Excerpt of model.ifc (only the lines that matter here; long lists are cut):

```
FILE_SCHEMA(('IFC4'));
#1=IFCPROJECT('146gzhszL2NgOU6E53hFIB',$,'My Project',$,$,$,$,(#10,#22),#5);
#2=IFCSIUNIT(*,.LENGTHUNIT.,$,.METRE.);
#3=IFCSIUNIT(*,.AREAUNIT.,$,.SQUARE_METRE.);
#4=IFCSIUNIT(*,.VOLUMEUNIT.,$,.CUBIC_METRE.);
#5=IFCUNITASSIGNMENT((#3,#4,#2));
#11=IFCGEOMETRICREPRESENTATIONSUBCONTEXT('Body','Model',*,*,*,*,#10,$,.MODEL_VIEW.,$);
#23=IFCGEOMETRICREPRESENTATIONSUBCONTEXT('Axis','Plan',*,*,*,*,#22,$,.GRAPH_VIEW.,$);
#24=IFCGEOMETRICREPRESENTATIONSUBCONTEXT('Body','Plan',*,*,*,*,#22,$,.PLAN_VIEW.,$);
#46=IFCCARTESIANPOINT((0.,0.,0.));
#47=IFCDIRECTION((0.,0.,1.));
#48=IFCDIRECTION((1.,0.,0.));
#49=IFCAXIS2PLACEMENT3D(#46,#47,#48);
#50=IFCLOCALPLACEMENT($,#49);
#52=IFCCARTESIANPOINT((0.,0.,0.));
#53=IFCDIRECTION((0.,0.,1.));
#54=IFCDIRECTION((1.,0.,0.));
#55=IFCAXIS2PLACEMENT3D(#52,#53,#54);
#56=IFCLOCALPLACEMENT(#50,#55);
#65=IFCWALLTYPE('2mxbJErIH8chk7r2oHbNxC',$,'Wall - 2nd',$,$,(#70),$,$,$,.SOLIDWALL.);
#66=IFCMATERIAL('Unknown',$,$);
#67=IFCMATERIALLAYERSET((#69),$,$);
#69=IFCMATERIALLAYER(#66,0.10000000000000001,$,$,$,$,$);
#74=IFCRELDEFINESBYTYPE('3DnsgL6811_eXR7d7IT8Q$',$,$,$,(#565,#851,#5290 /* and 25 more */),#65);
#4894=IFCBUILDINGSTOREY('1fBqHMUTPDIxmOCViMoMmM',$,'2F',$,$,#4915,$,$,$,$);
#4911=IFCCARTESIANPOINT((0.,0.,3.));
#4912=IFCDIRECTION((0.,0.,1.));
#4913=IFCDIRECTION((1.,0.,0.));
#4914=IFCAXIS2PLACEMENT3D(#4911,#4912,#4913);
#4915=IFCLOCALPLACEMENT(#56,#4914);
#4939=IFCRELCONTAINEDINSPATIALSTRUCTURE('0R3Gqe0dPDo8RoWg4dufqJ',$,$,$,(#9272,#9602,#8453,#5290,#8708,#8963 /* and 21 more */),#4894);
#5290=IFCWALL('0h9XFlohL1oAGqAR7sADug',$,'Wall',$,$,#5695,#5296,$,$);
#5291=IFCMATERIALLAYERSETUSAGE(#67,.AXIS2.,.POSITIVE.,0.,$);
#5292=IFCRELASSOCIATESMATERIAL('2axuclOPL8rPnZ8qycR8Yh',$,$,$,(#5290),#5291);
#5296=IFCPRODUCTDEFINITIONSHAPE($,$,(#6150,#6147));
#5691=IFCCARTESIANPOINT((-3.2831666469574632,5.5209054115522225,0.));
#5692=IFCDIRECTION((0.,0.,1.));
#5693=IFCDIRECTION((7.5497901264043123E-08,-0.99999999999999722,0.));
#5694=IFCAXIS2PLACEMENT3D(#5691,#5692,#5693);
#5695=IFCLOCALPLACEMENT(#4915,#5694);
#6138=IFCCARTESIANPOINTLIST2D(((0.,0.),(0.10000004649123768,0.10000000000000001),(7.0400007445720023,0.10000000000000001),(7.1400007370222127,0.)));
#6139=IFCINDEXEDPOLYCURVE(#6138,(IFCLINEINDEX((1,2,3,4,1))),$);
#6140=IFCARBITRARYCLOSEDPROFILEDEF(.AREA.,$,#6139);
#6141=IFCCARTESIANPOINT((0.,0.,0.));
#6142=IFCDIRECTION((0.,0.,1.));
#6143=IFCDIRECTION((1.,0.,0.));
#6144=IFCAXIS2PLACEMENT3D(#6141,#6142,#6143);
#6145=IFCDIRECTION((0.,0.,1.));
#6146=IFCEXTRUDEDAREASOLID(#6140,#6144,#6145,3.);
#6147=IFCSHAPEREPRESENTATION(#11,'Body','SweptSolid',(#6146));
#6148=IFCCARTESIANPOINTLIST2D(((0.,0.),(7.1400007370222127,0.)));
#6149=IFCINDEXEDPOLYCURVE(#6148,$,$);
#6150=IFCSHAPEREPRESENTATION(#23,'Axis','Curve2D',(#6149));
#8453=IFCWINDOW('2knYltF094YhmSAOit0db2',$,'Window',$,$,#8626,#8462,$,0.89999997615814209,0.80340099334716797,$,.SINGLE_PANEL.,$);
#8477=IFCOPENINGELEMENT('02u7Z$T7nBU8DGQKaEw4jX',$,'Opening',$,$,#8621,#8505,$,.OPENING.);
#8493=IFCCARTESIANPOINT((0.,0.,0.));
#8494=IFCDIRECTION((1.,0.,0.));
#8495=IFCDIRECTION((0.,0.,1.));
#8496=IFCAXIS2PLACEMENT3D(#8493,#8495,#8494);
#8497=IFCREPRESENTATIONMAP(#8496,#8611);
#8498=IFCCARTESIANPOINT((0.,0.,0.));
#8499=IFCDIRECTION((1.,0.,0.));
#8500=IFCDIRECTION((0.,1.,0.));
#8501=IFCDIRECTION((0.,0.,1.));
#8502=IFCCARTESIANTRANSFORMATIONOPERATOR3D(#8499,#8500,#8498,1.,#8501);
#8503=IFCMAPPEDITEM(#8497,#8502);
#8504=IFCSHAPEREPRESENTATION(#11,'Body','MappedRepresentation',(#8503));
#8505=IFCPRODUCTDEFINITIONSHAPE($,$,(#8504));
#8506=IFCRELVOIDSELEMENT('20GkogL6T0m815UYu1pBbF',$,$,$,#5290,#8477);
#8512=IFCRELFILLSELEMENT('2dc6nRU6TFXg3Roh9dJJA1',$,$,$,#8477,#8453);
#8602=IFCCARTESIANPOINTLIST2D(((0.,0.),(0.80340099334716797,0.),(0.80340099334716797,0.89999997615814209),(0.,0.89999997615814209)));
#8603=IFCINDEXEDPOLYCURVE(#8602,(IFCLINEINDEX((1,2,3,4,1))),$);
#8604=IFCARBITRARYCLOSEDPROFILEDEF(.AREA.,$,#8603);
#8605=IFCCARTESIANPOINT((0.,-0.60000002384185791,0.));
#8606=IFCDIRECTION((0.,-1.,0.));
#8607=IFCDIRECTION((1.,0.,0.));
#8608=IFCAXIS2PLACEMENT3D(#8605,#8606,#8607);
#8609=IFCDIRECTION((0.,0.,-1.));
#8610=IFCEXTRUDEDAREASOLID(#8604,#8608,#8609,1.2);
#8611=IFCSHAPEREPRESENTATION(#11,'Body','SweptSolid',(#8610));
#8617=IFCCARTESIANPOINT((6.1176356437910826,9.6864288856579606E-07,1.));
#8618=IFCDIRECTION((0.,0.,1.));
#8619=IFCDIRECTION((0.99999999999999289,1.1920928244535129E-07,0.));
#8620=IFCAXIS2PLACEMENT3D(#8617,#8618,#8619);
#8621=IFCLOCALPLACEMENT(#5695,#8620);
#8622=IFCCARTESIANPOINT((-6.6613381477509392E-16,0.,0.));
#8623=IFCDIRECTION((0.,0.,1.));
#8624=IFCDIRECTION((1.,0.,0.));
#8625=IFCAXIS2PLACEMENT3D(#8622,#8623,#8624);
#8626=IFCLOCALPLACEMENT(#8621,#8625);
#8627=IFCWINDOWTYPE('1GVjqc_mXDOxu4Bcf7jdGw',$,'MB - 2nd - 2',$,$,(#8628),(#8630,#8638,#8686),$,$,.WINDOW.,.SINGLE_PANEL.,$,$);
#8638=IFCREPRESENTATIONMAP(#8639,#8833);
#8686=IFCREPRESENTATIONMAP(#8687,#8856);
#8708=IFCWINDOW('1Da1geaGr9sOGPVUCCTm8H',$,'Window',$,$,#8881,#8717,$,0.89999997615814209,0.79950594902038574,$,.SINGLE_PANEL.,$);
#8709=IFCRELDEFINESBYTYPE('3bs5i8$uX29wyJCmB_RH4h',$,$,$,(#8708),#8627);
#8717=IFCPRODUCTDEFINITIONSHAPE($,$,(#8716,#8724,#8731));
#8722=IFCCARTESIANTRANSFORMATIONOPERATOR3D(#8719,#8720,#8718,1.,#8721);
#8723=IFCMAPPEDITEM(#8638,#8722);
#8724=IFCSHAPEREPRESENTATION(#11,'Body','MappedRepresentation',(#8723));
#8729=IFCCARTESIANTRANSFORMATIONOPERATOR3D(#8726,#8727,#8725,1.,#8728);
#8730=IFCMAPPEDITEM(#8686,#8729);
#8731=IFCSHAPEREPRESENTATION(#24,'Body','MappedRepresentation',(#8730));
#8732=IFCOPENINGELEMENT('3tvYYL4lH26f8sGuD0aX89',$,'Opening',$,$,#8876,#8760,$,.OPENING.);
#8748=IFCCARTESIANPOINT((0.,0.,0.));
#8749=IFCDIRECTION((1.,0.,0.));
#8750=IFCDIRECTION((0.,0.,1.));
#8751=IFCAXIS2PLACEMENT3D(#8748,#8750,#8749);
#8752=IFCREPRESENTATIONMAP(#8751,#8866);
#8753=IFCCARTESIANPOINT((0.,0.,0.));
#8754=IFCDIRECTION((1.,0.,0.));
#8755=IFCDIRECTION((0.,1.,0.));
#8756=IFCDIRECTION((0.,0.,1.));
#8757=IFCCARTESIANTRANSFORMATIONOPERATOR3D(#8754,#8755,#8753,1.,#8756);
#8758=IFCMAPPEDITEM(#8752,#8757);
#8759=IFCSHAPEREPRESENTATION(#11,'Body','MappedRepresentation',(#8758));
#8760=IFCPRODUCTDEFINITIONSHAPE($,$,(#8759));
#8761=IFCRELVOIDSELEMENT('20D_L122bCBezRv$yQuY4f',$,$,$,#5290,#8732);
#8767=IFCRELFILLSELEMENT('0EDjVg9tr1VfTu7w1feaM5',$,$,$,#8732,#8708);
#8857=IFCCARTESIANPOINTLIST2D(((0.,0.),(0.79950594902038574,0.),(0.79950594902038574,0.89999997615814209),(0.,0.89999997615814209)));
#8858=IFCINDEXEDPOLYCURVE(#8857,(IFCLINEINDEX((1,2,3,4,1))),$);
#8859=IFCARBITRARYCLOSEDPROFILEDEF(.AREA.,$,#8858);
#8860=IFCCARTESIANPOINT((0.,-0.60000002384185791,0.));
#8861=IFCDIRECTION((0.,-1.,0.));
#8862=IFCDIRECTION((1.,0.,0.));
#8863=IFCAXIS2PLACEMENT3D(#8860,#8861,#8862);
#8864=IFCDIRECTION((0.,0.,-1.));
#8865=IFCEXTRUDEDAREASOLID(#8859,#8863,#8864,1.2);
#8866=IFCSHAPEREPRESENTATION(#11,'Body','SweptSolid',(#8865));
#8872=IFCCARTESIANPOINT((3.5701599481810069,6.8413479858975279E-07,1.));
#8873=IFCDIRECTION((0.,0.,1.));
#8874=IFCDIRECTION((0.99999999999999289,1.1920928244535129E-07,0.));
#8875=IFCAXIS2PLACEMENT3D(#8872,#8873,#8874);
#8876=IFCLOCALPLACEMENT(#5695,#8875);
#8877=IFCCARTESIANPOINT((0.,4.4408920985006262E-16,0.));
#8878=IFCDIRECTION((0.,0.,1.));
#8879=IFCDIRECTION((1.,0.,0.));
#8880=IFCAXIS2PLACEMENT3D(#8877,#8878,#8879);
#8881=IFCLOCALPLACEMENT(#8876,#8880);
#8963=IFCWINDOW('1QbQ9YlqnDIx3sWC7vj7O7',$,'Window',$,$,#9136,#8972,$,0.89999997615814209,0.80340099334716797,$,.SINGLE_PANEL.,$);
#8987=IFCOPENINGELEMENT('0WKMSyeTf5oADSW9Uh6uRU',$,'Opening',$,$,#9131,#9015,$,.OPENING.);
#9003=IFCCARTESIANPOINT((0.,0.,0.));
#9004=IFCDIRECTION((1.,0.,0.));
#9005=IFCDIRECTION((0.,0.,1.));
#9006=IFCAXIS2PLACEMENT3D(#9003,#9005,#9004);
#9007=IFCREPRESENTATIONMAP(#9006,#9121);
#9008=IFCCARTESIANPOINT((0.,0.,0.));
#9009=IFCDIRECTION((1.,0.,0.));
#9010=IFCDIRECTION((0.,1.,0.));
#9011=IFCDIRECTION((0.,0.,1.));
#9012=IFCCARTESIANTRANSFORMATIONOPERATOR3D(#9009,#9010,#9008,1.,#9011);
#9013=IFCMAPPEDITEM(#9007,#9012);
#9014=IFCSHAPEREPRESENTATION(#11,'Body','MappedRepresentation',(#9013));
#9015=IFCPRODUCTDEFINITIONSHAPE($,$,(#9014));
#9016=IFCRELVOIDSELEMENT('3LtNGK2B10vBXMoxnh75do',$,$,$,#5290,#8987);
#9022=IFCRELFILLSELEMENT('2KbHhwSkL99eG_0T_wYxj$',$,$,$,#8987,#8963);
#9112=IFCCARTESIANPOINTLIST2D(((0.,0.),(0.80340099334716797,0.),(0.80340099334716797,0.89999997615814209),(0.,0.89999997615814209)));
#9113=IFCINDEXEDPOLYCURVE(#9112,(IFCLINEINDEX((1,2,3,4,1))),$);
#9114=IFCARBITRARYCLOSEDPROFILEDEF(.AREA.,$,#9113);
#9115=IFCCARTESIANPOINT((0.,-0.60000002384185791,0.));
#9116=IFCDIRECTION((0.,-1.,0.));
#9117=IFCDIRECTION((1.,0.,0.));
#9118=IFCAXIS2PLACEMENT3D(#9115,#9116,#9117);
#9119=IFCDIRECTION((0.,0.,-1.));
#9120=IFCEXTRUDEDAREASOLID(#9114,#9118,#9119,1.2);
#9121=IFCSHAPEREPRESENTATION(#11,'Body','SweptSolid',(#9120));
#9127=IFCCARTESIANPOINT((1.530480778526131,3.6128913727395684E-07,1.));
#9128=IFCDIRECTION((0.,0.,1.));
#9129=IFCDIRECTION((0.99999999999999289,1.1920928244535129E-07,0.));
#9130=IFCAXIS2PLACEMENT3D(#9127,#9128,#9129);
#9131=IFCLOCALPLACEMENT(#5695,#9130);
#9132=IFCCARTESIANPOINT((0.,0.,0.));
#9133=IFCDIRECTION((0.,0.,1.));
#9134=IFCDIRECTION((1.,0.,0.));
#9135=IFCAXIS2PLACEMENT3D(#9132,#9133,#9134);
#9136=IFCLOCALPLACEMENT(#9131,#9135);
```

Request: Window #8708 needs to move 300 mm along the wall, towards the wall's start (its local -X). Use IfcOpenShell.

```python
import ifcopenshell
import ifcopenshell.api.geometry
import ifcopenshell.util.placement
import ifcopenshell.util.unit

model = ifcopenshell.open("model.ifc")
unit_scale = ifcopenshell.util.unit.calculate_unit_scale(model)

window = model.by_guid("1Da1geaGr9sOGPVUCCTm8H")
opening = window.FillsVoids[0].RelatingOpeningElement
wall = opening.VoidsElements[0].RelatingBuildingElement

wall_matrix = ifcopenshell.util.placement.get_local_placement(wall.ObjectPlacement)
shift = wall_matrix[:3, 0] * -0.3 / unit_scale
before = ifcopenshell.util.placement.get_local_placement(window.ObjectPlacement)[:3, 3].copy()

# The window is placed relative to its opening, so it follows when the opening moves.
matrix = ifcopenshell.util.placement.get_local_placement(opening.ObjectPlacement)
matrix[:3, 3] += shift
ifcopenshell.api.geometry.edit_object_placement(
    model, product=opening, matrix=matrix, is_si=False, should_transform_children=True
)

after = ifcopenshell.util.placement.get_local_placement(window.ObjectPlacement)[:3, 3]
print("window moved by", (after - before).round(3) + 0.0)

model.write("model-out.ifc")
```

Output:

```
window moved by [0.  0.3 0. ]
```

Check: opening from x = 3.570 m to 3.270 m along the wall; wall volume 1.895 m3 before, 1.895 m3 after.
